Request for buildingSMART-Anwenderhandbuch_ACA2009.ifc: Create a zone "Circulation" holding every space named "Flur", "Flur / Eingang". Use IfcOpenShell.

First a look at what the model holds.

```python
import ifcopenshell

model = ifcopenshell.open("buildingSMART-Anwenderhandbuch_ACA2009.ifc")
print(model.schema)
seen = {}
for space in model.by_type("IfcSpace"):
    seen[space.LongName] = seen.get(space.LongName, 0) + 1
for name, count in sorted(seen.items(), key=str):
    print(count, "x", name)
print("zones:", [z.Name for z in model.by_type("IfcZone")][:20])
```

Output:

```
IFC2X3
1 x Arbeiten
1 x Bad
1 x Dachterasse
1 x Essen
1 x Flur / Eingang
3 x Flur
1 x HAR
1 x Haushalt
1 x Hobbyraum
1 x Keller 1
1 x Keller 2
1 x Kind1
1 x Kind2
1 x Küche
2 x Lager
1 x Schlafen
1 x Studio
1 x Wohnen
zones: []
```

```python
import ifcopenshell
import ifcopenshell.api.group
import ifcopenshell.api.root

model = ifcopenshell.open("buildingSMART-Anwenderhandbuch_ACA2009.ifc")

names = {"Flur", "Flur / Eingang"}
spaces = [s for s in model.by_type("IfcSpace") if s.LongName in names]

zone = ifcopenshell.api.root.create_entity(model, ifc_class="IfcZone", name="Circulation")
ifcopenshell.api.group.assign_group(model, products=spaces, group=zone)
print(len(spaces), "spaces in", zone.Name)

model.write("buildingSMART-Anwenderhandbuch_ACA2009_v2.ifc")
```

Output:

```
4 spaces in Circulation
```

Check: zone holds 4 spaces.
